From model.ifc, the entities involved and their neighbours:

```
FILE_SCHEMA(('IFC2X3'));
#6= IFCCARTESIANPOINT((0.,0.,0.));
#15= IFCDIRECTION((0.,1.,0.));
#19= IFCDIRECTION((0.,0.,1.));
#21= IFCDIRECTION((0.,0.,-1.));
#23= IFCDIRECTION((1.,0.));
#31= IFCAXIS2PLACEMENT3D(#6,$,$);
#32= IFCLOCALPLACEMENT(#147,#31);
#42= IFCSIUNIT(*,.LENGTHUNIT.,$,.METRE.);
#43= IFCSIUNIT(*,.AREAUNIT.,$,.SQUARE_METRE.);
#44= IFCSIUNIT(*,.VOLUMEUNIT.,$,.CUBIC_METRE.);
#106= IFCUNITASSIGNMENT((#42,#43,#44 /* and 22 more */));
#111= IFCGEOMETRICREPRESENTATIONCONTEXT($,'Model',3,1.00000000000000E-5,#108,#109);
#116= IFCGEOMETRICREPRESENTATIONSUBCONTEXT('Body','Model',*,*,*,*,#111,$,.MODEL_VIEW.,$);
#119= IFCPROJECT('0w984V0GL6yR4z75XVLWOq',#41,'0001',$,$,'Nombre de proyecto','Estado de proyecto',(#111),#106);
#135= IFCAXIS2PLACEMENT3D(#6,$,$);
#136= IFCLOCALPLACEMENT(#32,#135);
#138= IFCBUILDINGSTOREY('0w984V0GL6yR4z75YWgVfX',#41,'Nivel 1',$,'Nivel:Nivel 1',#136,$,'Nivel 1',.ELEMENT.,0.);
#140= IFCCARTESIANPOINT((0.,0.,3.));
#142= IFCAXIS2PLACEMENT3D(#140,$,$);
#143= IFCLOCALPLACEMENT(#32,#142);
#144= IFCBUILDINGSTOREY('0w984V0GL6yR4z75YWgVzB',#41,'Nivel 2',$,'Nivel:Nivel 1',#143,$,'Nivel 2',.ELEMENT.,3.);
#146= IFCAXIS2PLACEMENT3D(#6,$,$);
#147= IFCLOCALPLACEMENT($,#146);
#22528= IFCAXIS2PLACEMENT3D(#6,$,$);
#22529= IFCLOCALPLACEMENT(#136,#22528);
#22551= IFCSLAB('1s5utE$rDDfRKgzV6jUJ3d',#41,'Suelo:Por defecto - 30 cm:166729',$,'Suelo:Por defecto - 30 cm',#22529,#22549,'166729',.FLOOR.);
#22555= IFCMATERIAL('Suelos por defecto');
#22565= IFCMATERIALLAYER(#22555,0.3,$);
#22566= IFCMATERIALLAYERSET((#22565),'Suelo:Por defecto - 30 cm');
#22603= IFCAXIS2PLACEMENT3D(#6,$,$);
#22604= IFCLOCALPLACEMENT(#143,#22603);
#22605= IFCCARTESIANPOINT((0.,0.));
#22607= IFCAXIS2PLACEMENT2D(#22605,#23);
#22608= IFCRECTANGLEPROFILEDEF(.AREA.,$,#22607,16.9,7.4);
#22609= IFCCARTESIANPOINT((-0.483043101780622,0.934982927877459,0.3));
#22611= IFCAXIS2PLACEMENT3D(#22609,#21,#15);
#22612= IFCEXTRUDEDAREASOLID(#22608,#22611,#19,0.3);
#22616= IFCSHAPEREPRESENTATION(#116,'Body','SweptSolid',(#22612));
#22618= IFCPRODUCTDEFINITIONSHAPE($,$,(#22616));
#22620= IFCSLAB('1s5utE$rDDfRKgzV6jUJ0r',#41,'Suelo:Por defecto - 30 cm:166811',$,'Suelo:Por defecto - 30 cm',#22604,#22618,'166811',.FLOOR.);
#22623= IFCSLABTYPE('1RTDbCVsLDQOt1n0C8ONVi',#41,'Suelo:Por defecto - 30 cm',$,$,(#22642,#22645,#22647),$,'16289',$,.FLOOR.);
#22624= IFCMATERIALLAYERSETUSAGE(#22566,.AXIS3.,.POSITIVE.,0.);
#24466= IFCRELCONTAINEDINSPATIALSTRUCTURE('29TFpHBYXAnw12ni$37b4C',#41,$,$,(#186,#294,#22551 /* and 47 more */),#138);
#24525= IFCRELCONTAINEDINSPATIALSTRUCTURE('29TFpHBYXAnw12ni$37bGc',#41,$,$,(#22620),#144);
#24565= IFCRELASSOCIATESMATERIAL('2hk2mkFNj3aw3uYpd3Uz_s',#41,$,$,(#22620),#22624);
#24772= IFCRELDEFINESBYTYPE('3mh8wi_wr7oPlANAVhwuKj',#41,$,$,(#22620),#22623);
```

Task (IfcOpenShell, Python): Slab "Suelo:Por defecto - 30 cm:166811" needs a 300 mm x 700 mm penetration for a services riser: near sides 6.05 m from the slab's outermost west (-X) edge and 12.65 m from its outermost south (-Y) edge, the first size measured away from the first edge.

```python
import numpy as np
import ifcopenshell
import ifcopenshell.api.feature
import ifcopenshell.api.geometry
import ifcopenshell.api.root
import ifcopenshell.geom
import ifcopenshell.util.placement
import ifcopenshell.util.representation
import ifcopenshell.util.shape
import ifcopenshell.util.unit

model = ifcopenshell.open("model.ifc")
unit_scale = ifcopenshell.util.unit.calculate_unit_scale(model)
settings = ifcopenshell.geom.settings()


def volume(element):
    """Net volume in cubic metres, openings subtracted."""
    shape = ifcopenshell.geom.create_shape(settings, element)
    return ifcopenshell.util.shape.get_volume(shape.geometry)


slab = model.by_guid("1s5utE$rDDfRKgzV6jUJ0r")
before = volume(slab)

# Extent in the slab's own axes, in metres. The edges named are its -X and -Y sides.
slab_shape = ifcopenshell.geom.create_shape(settings, slab)
vertices = ifcopenshell.util.shape.get_vertices(slab_shape.geometry)
x_min, y_min, bottom = vertices.min(axis=0)
top = vertices[:, 2].max()

opening = ifcopenshell.api.root.create_entity(model, ifc_class="IfcOpeningElement", name="Services riser opening")
context = ifcopenshell.util.representation.get_context(model, "Model", "Body", "MODEL_VIEW")
width, depth = 0.3, 0.7
outline = [(0.0, 0.0), (width, 0.0), (width, depth), (0.0, depth), (0.0, 0.0)]
# Overshoot both faces by 50 mm so the cut is clean.
shape = ifcopenshell.api.geometry.add_slab_representation(
    model, context=context, depth=top - bottom + 0.1, polyline=outline
)
ifcopenshell.api.geometry.assign_representation(model, product=opening, representation=shape)

matrix = ifcopenshell.util.placement.get_local_placement(slab.ObjectPlacement)
matrix[:, 3] = matrix @ np.append(np.array([x_min + 6.05, y_min + 12.65, bottom - 0.05]) / unit_scale, 1.0)
ifcopenshell.api.geometry.edit_object_placement(model, product=opening, matrix=matrix, is_si=False)
ifcopenshell.api.feature.add_feature(model, feature=opening, element=slab)

after = volume(slab)

print(f"slab volume {before:.3f} -> {after:.3f} m3")

model.write("model_v2.ifc")
```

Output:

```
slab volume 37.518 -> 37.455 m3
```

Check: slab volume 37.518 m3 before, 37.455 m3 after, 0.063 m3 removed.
